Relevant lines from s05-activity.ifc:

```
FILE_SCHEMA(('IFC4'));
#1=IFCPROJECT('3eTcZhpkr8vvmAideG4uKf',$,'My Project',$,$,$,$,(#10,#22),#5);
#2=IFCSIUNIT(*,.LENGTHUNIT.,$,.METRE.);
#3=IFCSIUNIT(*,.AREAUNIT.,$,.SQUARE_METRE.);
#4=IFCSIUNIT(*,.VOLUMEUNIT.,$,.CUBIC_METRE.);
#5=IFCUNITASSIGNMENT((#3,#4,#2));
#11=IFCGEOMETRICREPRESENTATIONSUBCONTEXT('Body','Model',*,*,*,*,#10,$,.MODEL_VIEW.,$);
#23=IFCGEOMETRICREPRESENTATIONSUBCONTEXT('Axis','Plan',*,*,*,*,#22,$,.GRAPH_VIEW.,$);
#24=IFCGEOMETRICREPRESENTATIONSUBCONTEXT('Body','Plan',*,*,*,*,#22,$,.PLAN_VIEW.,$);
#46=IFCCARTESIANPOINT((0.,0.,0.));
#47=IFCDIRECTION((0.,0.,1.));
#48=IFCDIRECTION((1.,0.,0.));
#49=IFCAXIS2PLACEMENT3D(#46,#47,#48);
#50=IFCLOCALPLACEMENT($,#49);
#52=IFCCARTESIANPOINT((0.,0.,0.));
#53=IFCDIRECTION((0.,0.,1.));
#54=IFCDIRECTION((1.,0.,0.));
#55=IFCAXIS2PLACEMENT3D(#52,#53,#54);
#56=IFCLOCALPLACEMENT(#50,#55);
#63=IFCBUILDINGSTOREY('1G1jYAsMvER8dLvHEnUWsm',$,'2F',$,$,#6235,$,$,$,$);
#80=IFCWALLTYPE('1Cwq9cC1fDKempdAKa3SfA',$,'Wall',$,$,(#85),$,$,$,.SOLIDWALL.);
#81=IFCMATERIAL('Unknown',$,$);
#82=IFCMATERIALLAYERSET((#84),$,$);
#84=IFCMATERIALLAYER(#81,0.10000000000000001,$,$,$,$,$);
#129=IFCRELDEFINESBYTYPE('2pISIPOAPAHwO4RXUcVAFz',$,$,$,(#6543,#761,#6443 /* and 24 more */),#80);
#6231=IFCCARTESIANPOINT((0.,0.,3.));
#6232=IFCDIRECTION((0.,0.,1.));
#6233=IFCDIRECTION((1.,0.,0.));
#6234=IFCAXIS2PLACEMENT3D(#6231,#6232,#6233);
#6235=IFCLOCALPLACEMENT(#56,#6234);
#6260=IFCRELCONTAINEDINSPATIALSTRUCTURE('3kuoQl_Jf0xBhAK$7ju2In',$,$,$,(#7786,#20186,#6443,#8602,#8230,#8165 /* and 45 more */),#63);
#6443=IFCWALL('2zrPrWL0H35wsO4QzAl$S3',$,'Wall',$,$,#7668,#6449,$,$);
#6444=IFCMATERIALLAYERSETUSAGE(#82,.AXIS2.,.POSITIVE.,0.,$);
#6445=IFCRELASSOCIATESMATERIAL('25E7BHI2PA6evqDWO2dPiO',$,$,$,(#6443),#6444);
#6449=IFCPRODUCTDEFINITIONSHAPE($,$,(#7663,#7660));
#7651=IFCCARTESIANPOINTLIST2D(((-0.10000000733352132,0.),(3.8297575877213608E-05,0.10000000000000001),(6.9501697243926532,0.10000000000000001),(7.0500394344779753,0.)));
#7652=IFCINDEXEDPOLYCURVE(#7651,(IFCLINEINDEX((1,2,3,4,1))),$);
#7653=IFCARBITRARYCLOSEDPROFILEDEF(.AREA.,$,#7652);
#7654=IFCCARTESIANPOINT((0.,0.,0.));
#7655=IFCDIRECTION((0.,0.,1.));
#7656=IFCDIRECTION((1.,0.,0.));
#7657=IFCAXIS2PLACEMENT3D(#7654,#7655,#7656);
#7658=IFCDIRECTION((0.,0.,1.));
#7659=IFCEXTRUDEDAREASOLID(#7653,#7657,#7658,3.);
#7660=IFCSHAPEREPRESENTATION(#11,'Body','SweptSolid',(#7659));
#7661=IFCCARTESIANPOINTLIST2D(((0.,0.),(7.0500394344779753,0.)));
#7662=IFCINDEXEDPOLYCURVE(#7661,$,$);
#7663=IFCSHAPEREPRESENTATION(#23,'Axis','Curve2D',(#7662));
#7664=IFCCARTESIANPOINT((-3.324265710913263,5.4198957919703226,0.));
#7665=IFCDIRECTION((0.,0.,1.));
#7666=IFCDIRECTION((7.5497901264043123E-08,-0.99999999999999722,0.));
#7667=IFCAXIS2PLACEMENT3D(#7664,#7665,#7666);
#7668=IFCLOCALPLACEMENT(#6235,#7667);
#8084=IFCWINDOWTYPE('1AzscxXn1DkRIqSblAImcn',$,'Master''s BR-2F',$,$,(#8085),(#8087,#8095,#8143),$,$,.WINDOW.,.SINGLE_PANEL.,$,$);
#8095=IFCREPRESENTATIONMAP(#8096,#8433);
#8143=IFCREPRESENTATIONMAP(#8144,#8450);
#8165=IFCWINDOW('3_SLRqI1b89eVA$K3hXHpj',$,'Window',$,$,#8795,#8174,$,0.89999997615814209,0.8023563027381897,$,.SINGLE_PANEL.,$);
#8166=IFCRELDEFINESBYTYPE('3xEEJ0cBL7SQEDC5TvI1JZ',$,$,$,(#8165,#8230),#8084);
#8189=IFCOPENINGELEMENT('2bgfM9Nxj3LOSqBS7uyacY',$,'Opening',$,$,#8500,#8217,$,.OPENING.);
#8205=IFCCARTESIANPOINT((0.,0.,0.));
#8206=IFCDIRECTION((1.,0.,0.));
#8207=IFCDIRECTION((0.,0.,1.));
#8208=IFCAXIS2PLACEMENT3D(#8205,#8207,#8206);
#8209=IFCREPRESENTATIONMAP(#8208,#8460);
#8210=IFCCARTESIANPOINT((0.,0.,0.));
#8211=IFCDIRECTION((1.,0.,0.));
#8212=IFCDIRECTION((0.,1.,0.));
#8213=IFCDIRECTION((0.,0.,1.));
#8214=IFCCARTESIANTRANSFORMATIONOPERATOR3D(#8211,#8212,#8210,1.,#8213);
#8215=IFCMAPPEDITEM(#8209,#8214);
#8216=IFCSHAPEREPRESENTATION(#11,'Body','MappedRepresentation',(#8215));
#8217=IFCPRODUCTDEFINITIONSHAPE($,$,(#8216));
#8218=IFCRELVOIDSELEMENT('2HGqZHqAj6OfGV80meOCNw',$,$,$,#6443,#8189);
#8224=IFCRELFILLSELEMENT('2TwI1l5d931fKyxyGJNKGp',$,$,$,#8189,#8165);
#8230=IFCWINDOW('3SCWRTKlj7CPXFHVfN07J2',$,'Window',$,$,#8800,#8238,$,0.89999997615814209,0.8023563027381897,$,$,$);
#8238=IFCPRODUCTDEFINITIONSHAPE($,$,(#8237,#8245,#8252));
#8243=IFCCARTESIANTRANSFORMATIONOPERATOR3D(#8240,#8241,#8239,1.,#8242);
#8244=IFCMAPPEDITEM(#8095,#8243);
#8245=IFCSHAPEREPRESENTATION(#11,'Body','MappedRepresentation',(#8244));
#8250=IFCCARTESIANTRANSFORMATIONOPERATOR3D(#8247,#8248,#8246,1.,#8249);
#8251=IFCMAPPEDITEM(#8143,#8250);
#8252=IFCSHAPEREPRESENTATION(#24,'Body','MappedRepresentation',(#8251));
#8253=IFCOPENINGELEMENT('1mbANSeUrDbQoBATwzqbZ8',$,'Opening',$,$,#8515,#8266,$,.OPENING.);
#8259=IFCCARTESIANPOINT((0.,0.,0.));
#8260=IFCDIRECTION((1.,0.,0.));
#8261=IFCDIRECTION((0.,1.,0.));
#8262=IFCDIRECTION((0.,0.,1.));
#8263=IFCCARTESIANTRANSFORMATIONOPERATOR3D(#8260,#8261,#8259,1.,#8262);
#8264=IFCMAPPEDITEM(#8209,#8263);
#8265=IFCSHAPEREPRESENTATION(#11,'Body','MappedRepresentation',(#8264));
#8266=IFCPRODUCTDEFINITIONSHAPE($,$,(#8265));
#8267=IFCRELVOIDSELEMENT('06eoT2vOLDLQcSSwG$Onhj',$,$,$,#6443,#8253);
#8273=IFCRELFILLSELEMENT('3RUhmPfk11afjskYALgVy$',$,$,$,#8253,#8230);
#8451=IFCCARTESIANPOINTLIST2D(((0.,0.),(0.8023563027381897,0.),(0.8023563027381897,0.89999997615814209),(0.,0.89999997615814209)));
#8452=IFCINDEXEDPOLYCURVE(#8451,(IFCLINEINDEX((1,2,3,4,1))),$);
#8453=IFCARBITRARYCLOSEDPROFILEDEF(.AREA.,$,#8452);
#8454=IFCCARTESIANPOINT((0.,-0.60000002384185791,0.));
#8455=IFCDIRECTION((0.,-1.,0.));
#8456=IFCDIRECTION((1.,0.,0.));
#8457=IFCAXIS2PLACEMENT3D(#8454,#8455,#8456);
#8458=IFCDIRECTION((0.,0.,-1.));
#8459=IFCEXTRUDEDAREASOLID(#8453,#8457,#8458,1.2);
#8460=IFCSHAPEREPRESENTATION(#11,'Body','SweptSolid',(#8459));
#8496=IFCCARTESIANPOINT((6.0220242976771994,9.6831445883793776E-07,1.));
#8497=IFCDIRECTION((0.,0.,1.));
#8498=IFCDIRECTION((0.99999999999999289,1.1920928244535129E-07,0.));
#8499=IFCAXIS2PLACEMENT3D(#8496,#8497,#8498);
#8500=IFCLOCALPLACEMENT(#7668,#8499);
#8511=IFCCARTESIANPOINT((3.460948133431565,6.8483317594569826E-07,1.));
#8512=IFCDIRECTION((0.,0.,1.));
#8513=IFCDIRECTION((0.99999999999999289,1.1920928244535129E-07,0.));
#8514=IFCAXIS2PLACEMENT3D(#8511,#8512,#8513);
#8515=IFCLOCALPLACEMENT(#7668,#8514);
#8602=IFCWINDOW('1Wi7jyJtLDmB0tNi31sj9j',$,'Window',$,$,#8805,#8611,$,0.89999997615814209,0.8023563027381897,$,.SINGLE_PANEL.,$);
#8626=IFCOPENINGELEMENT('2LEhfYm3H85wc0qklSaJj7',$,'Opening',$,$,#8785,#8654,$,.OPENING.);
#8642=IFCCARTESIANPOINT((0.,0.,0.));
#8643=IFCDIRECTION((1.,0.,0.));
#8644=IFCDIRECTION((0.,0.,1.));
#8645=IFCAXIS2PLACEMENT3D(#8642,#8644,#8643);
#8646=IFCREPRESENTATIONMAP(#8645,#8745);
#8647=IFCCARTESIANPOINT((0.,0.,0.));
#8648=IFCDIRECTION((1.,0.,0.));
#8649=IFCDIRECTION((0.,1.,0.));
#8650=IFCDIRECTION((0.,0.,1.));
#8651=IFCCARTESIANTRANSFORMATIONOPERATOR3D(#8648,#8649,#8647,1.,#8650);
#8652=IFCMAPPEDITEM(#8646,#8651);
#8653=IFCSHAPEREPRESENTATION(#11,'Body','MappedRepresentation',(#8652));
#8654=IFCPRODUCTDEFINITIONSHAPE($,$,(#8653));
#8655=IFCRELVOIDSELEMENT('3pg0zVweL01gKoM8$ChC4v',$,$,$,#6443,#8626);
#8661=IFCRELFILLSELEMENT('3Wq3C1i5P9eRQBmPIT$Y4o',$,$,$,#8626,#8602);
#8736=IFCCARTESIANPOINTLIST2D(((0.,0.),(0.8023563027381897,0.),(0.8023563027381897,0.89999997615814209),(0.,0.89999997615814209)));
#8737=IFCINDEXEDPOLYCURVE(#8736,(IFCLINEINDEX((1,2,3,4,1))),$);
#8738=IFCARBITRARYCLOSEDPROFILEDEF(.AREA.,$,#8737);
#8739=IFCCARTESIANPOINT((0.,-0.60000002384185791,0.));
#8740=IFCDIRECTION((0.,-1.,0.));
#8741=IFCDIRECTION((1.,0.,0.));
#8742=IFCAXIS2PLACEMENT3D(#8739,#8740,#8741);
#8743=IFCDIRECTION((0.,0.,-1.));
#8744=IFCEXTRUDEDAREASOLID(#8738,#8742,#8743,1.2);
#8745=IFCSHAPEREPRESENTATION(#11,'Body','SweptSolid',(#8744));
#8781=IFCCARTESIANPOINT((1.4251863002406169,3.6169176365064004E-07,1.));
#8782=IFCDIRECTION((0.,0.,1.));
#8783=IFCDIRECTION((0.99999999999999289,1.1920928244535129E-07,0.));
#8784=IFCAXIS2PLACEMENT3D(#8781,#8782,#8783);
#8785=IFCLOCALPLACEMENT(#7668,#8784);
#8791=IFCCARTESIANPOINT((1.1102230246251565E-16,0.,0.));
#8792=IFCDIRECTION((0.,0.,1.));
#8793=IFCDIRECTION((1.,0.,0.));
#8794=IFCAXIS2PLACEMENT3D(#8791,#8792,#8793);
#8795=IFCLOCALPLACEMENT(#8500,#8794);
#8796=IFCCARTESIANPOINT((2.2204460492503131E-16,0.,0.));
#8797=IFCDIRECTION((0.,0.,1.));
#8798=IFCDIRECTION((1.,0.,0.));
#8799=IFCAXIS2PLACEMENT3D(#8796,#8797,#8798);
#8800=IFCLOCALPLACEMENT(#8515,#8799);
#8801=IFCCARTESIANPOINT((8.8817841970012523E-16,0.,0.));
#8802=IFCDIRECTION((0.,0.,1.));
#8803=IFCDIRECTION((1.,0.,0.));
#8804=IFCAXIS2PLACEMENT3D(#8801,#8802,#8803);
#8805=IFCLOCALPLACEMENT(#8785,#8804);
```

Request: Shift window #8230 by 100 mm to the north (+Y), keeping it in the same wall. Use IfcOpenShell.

```python
import ifcopenshell
import ifcopenshell.api.geometry
import ifcopenshell.util.placement
import ifcopenshell.util.unit

model = ifcopenshell.open("s05-activity.ifc")
unit_scale = ifcopenshell.util.unit.calculate_unit_scale(model)

window = model.by_guid("3SCWRTKlj7CPXFHVfN07J2")
opening = window.FillsVoids[0].RelatingOpeningElement
wall = opening.VoidsElements[0].RelatingBuildingElement

wall_matrix = ifcopenshell.util.placement.get_local_placement(wall.ObjectPlacement)
shift = wall_matrix[:3, 0] * -0.1 / unit_scale
before = ifcopenshell.util.placement.get_local_placement(window.ObjectPlacement)[:3, 3].copy()

# The window is placed relative to its opening, so it follows when the opening moves.
matrix = ifcopenshell.util.placement.get_local_placement(opening.ObjectPlacement)
matrix[:3, 3] += shift
ifcopenshell.api.geometry.edit_object_placement(
    model, product=opening, matrix=matrix, is_si=False, should_transform_children=True
)

after = ifcopenshell.util.placement.get_local_placement(window.ObjectPlacement)[:3, 3]
print("window moved by", (after - before).round(3) + 0.0)

model.write("s05-activity_edited.ifc")
```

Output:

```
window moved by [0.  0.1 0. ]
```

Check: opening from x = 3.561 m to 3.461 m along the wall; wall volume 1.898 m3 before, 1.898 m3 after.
